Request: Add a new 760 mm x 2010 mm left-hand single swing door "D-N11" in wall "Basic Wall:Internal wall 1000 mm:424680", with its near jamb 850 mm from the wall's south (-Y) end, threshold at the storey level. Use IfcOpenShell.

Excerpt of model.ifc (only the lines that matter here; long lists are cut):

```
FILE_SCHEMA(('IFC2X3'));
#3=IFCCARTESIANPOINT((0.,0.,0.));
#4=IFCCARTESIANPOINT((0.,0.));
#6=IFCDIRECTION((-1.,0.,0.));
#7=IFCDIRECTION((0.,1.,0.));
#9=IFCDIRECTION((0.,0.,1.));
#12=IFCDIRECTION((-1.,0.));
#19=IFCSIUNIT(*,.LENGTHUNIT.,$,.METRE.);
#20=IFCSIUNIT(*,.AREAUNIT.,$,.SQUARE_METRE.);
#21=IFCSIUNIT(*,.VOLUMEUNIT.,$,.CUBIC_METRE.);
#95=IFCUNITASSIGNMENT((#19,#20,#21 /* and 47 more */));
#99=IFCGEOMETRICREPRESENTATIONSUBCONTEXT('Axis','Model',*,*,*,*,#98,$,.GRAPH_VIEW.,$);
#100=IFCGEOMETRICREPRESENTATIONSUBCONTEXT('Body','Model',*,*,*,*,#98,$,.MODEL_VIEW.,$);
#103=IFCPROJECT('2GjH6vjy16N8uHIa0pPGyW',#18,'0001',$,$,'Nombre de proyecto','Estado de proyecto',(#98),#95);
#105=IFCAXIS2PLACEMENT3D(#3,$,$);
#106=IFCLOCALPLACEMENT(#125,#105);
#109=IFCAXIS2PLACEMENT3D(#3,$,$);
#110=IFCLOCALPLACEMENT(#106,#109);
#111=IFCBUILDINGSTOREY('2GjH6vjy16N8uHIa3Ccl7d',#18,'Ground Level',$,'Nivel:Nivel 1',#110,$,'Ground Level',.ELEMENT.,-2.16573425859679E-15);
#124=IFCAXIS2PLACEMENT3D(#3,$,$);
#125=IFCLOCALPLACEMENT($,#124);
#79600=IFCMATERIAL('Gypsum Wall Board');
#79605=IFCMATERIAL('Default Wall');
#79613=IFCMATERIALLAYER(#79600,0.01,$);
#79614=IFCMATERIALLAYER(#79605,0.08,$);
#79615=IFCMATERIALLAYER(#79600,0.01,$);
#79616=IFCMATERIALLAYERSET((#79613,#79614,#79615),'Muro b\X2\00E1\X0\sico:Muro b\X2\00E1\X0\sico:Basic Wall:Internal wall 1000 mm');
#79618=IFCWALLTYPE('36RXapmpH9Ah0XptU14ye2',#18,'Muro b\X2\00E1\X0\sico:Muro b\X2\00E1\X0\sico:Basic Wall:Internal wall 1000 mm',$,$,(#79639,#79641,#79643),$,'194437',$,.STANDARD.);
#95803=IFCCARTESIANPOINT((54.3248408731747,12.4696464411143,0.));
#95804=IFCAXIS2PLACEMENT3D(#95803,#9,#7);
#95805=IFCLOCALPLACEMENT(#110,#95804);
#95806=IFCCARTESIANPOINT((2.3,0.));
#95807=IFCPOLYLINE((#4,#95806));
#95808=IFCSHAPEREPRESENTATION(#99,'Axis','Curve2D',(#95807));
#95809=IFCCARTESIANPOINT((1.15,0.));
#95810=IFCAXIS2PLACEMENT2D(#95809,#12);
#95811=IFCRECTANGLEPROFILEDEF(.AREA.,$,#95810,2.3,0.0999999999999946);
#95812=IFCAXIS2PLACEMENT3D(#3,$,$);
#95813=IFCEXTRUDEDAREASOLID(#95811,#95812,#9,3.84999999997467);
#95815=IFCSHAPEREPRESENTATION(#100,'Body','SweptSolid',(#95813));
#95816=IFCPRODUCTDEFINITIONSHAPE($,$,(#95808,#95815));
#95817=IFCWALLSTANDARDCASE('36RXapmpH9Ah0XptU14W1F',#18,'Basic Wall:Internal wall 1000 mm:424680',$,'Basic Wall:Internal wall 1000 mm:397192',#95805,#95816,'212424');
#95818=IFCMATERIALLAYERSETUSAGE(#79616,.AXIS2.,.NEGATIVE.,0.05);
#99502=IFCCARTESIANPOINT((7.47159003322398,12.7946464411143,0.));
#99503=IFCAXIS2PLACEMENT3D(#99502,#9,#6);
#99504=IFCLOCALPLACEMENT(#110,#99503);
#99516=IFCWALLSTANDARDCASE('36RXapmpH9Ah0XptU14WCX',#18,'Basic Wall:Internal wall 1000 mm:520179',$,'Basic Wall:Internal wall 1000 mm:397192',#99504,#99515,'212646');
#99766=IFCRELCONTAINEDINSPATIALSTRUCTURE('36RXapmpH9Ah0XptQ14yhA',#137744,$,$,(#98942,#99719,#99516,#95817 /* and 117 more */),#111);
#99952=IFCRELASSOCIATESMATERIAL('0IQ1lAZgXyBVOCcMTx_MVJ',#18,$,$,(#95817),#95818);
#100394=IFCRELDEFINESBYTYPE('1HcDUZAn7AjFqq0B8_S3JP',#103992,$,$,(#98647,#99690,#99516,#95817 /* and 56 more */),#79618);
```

```python
import numpy as np
import ifcopenshell
import ifcopenshell.api.feature
import ifcopenshell.api.geometry
import ifcopenshell.api.root
import ifcopenshell.api.spatial
import ifcopenshell.api.type
import ifcopenshell.geom
import ifcopenshell.util.element
import ifcopenshell.util.placement
import ifcopenshell.util.representation
import ifcopenshell.util.shape
import ifcopenshell.util.unit

model = ifcopenshell.open("model.ifc")
unit_scale = ifcopenshell.util.unit.calculate_unit_scale(model)
settings = ifcopenshell.geom.settings()


def volume(element):
    """Net volume in cubic metres, openings subtracted."""
    shape = ifcopenshell.geom.create_shape(settings, element)
    return ifcopenshell.util.shape.get_volume(shape.geometry)


wall = model.by_guid("36RXapmpH9Ah0XptU14W1F")
storey = ifcopenshell.util.element.get_container(wall, ifc_class="IfcBuildingStorey")
context = ifcopenshell.util.representation.get_context(model, "Model", "Body", "MODEL_VIEW")
before = volume(wall)

width, height, from_end, sill = 0.76, 2.01, 0.85, 0.0  # metres

# The wall runs along its own X axis, and the end named is its -X end.
wall_shape = ifcopenshell.geom.create_shape(settings, wall)
x, y, z = ifcopenshell.util.shape.get_vertices(wall_shape.geometry).T
start = x.min() + from_end
face, thickness = float(y.min()), float(y.max() - y.min())
wall_matrix = ifcopenshell.util.placement.get_local_placement(wall.ObjectPlacement)
level = ifcopenshell.util.placement.get_local_placement(storey.ObjectPlacement)[2, 3]


def in_wall(x, y):
    """Placement at x, y metres in the wall's axes, at sill height."""
    matrix = wall_matrix.copy()
    matrix[:, 3] = wall_matrix @ np.array([x / unit_scale, y / unit_scale, 0.0, 1.0])
    matrix[2, 3] = level + sill / unit_scale
    return matrix


# Opening: a box that overshoots both wall faces by 50 mm.
opening = ifcopenshell.api.root.create_entity(model, ifc_class="IfcOpeningElement")
box = ifcopenshell.api.geometry.add_wall_representation(
    model, context=context, length=width, height=height, thickness=thickness + 0.1
)
ifcopenshell.api.geometry.assign_representation(model, product=opening, representation=box)
ifcopenshell.api.geometry.edit_object_placement(model, product=opening, matrix=in_wall(start, face - 0.05), is_si=False)
ifcopenshell.api.feature.add_feature(model, feature=opening, element=wall)

door = ifcopenshell.api.root.create_entity(model, ifc_class="IfcDoor", name="D-N11")
door.OverallWidth, door.OverallHeight = width / unit_scale, height / unit_scale
body = ifcopenshell.api.geometry.add_door_representation(
    model,
    context=context,
    overall_width=door.OverallWidth,
    overall_height=door.OverallHeight,
    operation_type="SINGLE_SWING_LEFT",
    lining_properties={"LiningDepth": thickness / unit_scale, "ThresholdDepth": thickness / unit_scale},
)
ifcopenshell.api.geometry.assign_representation(model, product=door, representation=body)
ifcopenshell.api.spatial.assign_container(model, products=[door], relating_structure=storey)
fills = ifcopenshell.api.feature.add_filling(model, opening=opening, element=door)
fills.OwnerHistory = door.OwnerHistory  # required in IFC2X3

# IFC2X3 keeps the operation on the door style.
style = ifcopenshell.api.root.create_entity(model, ifc_class="IfcDoorStyle", name="D-N11")
style.OperationType, style.ConstructionType = "SINGLE_SWING_LEFT", "NOTDEFINED"
style.ParameterTakesPrecedence = style.Sizeable = False
ifcopenshell.api.type.assign_type(model, related_objects=[door], relating_type=style)

# The lining spans the wall, so the door starts at the wall face.
ifcopenshell.api.geometry.edit_object_placement(model, product=door, matrix=in_wall(start, face), is_si=False)

after = volume(wall)

print(f"wall volume {before:.3f} -> {after:.3f} m3")

model.write("model_v2.ifc")
```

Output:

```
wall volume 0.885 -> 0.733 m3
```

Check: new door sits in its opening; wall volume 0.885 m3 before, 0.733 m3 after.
